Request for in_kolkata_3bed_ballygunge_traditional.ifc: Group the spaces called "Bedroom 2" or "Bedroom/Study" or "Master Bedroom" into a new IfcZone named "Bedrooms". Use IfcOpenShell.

First a look at what the model holds.

```python
import ifcopenshell

model = ifcopenshell.open("in_kolkata_3bed_ballygunge_traditional.ifc")
print(model.schema)
seen = {}
for space in model.by_type("IfcSpace"):
    seen[space.LongName] = seen.get(space.LongName, 0) + 1
for name, count in sorted(seen.items(), key=str):
    print(count, "x", name)
print("zones:", [z.Name for z in model.by_type("IfcZone")][:20])
```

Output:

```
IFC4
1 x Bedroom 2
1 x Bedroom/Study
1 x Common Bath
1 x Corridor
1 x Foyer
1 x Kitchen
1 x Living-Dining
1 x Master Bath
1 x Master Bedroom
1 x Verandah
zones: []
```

```python
import ifcopenshell
import ifcopenshell.api.group
import ifcopenshell.api.root

model = ifcopenshell.open("in_kolkata_3bed_ballygunge_traditional.ifc")

names = {"Bedroom 2", "Bedroom/Study", "Master Bedroom"}
spaces = [s for s in model.by_type("IfcSpace") if s.LongName in names]

zone = ifcopenshell.api.root.create_entity(model, ifc_class="IfcZone", name="Bedrooms")
ifcopenshell.api.group.assign_group(model, products=spaces, group=zone)
print(len(spaces), "spaces in", zone.Name)

model.write("in_kolkata_3bed_ballygunge_traditional_updated.ifc")
```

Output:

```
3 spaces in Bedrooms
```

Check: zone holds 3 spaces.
